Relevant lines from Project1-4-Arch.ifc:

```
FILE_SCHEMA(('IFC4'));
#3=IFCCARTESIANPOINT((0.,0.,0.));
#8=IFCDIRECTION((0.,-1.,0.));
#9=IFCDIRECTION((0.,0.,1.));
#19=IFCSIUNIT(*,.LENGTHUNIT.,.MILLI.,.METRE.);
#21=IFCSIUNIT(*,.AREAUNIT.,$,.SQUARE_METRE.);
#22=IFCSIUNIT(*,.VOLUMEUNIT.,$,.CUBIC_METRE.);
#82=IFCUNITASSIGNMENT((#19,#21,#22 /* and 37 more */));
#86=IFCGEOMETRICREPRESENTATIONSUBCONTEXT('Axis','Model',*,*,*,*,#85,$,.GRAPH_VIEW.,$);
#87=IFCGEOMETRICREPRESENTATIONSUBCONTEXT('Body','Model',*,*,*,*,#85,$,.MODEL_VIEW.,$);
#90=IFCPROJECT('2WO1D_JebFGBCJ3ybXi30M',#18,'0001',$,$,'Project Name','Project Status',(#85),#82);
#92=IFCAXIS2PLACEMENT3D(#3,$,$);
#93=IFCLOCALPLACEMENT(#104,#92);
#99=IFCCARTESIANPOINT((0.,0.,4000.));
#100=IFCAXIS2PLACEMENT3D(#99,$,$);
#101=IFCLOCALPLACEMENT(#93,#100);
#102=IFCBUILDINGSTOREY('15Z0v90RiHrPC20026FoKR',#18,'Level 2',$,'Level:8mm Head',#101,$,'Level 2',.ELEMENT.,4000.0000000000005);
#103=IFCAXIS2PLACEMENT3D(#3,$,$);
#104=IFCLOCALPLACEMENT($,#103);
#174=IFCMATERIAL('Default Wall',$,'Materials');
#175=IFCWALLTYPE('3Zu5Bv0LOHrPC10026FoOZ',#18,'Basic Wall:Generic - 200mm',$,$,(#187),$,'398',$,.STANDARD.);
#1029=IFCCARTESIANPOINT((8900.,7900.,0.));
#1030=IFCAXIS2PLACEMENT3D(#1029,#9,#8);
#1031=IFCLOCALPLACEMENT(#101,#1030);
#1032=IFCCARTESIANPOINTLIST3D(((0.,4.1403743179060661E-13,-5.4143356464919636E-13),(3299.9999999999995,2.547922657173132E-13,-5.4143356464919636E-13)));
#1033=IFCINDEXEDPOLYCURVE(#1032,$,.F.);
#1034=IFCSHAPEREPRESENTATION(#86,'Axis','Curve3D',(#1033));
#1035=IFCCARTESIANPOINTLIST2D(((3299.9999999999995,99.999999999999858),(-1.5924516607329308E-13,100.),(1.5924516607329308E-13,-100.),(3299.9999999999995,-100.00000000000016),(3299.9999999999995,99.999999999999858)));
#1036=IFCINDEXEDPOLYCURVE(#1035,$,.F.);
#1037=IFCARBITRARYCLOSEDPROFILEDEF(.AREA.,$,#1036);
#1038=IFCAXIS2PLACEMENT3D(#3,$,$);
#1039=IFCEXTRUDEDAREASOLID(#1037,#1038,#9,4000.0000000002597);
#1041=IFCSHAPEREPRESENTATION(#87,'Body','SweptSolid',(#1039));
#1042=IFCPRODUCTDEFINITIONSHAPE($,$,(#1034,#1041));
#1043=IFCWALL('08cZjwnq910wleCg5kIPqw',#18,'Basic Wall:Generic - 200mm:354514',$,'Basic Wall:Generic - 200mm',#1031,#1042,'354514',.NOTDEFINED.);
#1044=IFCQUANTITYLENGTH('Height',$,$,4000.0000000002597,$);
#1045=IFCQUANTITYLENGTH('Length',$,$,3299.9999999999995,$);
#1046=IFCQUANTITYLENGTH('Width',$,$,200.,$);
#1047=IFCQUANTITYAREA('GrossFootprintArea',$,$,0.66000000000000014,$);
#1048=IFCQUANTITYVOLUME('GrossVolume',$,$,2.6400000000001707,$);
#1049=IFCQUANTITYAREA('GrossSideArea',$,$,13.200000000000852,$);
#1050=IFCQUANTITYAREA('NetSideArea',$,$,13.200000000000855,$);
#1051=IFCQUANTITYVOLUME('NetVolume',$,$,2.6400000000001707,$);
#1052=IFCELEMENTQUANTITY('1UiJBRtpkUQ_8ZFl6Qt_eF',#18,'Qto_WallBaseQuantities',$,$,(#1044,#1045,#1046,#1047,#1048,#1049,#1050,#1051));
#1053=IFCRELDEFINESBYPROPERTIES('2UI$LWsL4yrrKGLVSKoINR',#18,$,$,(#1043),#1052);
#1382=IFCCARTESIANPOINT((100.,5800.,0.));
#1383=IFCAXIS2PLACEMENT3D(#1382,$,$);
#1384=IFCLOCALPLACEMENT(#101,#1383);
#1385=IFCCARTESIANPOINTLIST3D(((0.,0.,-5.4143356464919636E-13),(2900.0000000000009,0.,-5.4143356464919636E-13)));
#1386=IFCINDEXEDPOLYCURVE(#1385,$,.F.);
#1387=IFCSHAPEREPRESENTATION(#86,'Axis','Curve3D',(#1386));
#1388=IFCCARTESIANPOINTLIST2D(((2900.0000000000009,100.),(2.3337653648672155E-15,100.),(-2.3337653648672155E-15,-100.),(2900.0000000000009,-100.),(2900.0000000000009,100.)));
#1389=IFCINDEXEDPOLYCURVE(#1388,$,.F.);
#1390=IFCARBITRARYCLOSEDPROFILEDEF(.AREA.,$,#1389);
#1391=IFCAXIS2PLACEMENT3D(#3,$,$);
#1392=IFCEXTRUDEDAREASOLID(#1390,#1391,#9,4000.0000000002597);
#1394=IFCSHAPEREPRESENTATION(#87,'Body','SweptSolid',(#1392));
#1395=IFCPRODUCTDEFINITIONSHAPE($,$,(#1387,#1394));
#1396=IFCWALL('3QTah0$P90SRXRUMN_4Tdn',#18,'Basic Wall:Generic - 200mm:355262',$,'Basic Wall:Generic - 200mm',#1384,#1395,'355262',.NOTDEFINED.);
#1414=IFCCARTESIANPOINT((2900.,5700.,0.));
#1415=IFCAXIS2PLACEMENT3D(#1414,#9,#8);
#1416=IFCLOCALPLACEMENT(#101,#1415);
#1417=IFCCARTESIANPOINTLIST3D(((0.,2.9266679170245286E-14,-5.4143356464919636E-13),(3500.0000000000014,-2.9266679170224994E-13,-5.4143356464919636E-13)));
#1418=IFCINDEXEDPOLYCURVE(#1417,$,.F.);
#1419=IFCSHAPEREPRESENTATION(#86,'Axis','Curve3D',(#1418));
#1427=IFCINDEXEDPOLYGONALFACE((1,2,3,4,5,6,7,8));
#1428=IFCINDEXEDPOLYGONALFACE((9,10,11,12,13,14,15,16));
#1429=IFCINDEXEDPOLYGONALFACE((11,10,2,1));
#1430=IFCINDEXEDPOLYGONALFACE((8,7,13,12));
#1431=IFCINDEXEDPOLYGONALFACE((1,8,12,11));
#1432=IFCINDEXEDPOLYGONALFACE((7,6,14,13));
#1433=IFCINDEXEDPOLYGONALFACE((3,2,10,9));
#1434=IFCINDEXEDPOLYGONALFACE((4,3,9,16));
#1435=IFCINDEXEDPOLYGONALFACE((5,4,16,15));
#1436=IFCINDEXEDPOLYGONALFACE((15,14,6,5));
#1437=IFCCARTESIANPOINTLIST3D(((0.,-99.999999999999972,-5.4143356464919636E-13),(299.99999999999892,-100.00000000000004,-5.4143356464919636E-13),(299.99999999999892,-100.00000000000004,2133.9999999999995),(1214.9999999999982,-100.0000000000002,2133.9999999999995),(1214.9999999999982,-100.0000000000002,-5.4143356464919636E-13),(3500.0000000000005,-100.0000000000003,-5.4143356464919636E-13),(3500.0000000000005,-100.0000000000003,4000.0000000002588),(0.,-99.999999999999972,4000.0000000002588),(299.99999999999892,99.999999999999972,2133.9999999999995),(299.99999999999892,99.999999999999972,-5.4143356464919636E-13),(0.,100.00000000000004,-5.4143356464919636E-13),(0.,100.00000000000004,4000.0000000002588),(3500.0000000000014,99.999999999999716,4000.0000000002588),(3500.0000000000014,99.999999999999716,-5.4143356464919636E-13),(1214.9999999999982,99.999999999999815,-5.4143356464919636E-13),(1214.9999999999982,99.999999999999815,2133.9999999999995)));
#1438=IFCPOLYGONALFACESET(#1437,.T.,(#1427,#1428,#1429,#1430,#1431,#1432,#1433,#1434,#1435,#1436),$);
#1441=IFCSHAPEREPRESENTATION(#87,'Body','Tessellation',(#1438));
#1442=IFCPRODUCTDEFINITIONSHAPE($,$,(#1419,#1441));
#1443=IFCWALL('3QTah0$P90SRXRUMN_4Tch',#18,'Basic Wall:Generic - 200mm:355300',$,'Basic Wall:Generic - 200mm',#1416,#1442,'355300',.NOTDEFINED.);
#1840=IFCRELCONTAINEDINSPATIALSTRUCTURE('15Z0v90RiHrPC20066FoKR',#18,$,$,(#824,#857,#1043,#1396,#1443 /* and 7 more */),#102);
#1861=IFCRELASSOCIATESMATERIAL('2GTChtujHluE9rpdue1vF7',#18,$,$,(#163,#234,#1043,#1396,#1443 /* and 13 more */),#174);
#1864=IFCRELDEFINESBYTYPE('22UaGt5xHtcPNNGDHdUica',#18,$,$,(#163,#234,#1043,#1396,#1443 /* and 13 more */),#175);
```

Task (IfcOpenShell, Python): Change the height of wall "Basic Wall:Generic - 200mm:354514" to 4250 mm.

```python
import ifcopenshell
import ifcopenshell.api.pset
import ifcopenshell.geom
import ifcopenshell.util.element
import ifcopenshell.util.representation
import ifcopenshell.util.shape
import ifcopenshell.util.unit

model = ifcopenshell.open("Project1-4-Arch.ifc")
unit_scale = ifcopenshell.util.unit.calculate_unit_scale(model)
area_scale = ifcopenshell.util.unit.calculate_unit_scale(model, "AREAUNIT")
volume_scale = ifcopenshell.util.unit.calculate_unit_scale(model, "VOLUMEUNIT")
settings = ifcopenshell.geom.settings()


def volume(element):
    """Net volume in cubic metres, openings subtracted."""
    shape = ifcopenshell.geom.create_shape(settings, element)
    return ifcopenshell.util.shape.get_volume(shape.geometry)


wall = model.by_id(1043)
before = volume(wall)

body = ifcopenshell.util.representation.get_representation(wall, "Model", "Body")
solid = body.Items[0]
old_height = solid.Depth
solid.Depth = 4.25 / unit_scale
after = volume(wall)
thickness = 0.2  # wall thickness in metres

# Update the stored height, areas and volumes.
qto = model.by_id(ifcopenshell.util.element.get_pset(wall, "Qto_WallBaseQuantities", should_inherit=False)["id"])
ifcopenshell.api.pset.edit_qto(model, qto=qto, properties={
    "Height": solid.Depth,
    "GrossVolume": ifcopenshell.util.element.get_pset(wall, "Qto_WallBaseQuantities", "GrossVolume") * solid.Depth / old_height,
    "GrossSideArea": ifcopenshell.util.element.get_pset(wall, "Qto_WallBaseQuantities", "GrossSideArea") * solid.Depth / old_height,
    "NetSideArea": after / thickness / area_scale,
    "NetVolume": after / volume_scale,
})

print(f"height {old_height:g} -> {solid.Depth:g}, volume {before:.3f} -> {after:.3f} m3")

model.write("Project1-4-Arch_updated.ifc")
```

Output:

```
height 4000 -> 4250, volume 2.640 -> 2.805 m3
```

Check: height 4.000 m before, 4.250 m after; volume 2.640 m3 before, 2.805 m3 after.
